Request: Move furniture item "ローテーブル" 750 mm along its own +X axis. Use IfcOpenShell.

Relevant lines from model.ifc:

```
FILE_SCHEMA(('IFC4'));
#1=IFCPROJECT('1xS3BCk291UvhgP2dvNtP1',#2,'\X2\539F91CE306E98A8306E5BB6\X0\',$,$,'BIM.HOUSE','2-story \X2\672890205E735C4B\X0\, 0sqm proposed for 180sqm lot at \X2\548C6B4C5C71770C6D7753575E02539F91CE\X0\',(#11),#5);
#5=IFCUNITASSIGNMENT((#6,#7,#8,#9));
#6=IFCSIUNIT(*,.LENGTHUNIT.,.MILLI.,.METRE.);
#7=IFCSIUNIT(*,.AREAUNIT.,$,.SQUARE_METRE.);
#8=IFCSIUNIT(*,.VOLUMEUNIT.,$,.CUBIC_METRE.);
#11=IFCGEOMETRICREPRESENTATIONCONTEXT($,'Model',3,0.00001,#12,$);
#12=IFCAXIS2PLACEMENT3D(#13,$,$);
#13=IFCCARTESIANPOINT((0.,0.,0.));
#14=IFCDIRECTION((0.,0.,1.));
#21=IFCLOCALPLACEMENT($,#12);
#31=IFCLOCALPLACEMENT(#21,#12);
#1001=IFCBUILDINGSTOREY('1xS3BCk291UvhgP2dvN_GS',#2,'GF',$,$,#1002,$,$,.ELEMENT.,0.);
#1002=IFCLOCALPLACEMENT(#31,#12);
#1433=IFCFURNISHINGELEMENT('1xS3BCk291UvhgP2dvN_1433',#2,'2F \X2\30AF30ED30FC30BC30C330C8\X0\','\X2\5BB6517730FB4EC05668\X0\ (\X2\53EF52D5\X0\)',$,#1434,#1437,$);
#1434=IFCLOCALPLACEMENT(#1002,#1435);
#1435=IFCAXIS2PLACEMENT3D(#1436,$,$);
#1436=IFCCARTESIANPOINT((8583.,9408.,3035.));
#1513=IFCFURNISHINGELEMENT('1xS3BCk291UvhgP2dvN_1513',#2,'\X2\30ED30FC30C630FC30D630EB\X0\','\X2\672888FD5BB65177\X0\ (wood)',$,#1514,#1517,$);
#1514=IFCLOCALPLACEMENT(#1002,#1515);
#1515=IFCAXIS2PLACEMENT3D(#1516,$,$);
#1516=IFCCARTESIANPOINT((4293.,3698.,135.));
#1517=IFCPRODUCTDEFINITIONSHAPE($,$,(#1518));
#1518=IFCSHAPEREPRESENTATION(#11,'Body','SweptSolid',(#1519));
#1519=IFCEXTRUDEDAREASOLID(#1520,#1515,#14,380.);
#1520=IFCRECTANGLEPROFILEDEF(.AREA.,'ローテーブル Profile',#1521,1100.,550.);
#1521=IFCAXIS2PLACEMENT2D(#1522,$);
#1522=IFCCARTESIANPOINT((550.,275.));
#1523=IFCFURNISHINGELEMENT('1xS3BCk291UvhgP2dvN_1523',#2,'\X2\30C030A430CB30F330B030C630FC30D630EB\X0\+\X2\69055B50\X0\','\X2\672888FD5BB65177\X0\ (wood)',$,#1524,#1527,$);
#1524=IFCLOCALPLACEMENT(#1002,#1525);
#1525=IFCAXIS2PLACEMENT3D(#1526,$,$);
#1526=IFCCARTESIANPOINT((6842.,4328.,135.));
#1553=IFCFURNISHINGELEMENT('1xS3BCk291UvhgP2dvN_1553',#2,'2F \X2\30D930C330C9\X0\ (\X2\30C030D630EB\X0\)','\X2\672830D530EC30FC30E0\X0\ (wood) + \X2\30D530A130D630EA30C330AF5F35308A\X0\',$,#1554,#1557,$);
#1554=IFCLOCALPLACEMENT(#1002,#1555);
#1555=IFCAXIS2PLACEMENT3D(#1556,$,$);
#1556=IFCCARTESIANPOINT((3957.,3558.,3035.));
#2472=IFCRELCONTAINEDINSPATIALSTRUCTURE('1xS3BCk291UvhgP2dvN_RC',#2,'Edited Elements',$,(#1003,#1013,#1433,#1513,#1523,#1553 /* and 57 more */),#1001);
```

```python
import ifcopenshell
import ifcopenshell.api.geometry
import ifcopenshell.util.placement
import ifcopenshell.util.unit

model = ifcopenshell.open("model.ifc")
unit_scale = ifcopenshell.util.unit.calculate_unit_scale(model)

item = model.by_guid("1xS3BCk291UvhgP2dvN_1513")
matrix = ifcopenshell.util.placement.get_local_placement(item.ObjectPlacement)
matrix[:3, 3] += matrix[:3, 0] * 0.75 / unit_scale
ifcopenshell.api.geometry.edit_object_placement(model, product=item, matrix=matrix, is_si=False)

print(ifcopenshell.util.placement.get_local_placement(item.ObjectPlacement).round(3) + 0.0)

model.write("model_updated.ifc")
```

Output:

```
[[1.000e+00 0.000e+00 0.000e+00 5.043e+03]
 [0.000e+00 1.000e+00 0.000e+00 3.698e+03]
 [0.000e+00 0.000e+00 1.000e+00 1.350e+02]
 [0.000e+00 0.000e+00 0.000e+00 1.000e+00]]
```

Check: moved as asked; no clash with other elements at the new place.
